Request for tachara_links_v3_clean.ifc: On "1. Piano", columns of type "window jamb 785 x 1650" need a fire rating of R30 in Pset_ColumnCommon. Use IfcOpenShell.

First a look at what the model holds.

```python
import ifcopenshell
import ifcopenshell.util.element

model = ifcopenshell.open("tachara_links_v3_clean.ifc")
print(model.schema)
storey = next(s for s in model.by_type("IfcBuildingStorey") if s.Name == "1. Piano")
columns = [e for e in ifcopenshell.util.element.get_decomposition(storey) if e.is_a("IfcColumn")]
seen = {}
for e in columns:
    element_type = ifcopenshell.util.element.get_type(e)
    key = (element_type.Name if element_type != e and element_type else None, ifcopenshell.util.element.get_pset(e, "Pset_ColumnCommon", "FireRating"))
    seen[key] = seen.get(key, 0) + 1
for (name, value), count in sorted(seen.items(), key=str):
    print(count, "x", name, "|", value)
```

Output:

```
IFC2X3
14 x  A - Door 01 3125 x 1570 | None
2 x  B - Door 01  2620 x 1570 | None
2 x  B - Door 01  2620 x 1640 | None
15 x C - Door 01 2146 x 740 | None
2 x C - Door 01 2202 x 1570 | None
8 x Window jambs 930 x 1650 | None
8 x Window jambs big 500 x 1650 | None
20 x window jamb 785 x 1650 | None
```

```python
import ifcopenshell
import ifcopenshell.api.pset
import ifcopenshell.util.element

model = ifcopenshell.open("tachara_links_v3_clean.ifc")

storey = next(s for s in model.by_type("IfcBuildingStorey") if s.Name == "1. Piano")
columns = [e for e in ifcopenshell.util.element.get_decomposition(storey) if e.is_a("IfcColumn")]

count = 0
for e in columns:
    element_type = ifcopenshell.util.element.get_type(e)
    if element_type in (None, e) or element_type.Name != "window jamb 785 x 1650":
        continue
    # add_pset returns the element's existing set when there is one.
    pset = ifcopenshell.api.pset.add_pset(model, product=e, name="Pset_ColumnCommon")
    ifcopenshell.api.pset.edit_pset(model, pset=pset, properties={"FireRating": "R30"})
    count += 1

print(count, "columns updated")

model.write("tachara_links_v3_clean_edited.ifc")
```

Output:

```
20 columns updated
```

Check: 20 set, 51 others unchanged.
